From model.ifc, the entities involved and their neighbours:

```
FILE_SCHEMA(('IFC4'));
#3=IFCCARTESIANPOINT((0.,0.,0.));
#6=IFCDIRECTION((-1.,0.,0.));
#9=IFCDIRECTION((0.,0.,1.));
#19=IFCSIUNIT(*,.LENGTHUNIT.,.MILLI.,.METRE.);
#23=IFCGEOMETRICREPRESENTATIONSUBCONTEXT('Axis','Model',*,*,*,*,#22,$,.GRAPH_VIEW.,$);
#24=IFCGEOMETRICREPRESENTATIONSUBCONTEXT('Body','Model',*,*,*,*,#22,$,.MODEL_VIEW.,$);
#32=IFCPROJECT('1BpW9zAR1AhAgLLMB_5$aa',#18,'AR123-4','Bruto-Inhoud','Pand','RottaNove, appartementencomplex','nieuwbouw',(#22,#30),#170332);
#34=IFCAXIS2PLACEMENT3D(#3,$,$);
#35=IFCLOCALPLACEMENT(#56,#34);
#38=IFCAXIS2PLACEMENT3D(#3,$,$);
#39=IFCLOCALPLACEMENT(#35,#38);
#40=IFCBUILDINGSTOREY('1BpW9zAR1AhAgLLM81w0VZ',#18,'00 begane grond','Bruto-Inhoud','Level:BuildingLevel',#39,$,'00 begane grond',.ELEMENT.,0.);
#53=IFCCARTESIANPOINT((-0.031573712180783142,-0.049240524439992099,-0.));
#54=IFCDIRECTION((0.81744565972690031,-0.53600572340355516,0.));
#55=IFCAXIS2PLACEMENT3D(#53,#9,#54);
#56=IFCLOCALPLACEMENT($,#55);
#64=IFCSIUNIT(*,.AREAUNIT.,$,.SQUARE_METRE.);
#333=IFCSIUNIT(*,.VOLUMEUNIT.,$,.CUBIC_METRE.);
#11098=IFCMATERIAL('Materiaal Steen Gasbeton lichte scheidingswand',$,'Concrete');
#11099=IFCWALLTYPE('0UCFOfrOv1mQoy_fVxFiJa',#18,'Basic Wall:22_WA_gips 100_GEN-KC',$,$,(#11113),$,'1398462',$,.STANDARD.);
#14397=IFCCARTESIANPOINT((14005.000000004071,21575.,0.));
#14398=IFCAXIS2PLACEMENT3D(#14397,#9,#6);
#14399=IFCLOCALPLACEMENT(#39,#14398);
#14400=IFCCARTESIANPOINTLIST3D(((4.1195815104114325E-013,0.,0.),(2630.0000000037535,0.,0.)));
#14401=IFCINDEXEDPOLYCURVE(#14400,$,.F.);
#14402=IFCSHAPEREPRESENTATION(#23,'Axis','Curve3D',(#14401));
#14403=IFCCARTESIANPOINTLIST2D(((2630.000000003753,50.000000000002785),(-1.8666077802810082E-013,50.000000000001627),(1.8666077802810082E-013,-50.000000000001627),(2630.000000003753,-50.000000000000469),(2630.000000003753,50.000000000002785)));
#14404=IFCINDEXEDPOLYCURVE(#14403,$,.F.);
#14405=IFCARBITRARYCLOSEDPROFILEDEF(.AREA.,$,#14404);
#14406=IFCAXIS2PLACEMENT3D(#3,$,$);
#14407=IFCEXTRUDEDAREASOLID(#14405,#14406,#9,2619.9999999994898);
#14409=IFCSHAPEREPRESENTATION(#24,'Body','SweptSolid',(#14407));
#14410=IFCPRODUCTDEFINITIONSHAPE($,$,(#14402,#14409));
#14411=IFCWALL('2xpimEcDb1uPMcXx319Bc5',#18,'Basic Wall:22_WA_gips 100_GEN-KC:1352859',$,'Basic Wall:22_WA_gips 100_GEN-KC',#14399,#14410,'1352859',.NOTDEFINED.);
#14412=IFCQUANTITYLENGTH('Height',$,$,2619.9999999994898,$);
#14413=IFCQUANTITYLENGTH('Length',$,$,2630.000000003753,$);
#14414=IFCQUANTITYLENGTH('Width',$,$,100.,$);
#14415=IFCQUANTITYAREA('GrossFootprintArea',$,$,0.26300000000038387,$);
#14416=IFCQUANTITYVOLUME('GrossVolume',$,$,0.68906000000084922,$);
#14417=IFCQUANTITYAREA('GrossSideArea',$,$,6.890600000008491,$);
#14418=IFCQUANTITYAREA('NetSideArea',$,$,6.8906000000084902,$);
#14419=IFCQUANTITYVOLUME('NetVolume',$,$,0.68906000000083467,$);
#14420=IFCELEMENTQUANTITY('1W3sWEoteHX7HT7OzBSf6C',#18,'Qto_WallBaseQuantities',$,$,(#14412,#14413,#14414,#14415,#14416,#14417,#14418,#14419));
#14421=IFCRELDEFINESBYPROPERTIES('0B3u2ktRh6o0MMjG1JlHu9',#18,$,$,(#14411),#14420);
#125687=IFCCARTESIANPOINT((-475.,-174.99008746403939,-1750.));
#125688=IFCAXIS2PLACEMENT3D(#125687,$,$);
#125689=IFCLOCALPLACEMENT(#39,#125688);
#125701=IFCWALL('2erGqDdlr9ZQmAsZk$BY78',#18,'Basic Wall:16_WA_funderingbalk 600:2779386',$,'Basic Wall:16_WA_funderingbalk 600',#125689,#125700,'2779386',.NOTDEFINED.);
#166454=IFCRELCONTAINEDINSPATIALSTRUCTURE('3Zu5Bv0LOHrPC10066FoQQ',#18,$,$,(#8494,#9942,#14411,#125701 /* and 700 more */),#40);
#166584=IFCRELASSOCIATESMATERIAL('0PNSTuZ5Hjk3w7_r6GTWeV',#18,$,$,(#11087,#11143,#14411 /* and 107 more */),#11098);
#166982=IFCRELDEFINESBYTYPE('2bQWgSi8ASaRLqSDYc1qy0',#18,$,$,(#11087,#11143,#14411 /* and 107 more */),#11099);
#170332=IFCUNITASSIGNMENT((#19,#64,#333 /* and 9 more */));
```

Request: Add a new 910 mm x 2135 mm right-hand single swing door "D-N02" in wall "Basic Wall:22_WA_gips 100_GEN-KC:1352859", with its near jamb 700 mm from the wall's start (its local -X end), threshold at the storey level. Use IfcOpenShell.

```python
import numpy as np
import ifcopenshell
import ifcopenshell.api.feature
import ifcopenshell.api.geometry
import ifcopenshell.api.pset
import ifcopenshell.api.root
import ifcopenshell.api.spatial
import ifcopenshell.geom
import ifcopenshell.util.element
import ifcopenshell.util.placement
import ifcopenshell.util.representation
import ifcopenshell.util.shape
import ifcopenshell.util.unit

model = ifcopenshell.open("model.ifc")
unit_scale = ifcopenshell.util.unit.calculate_unit_scale(model)
area_scale = ifcopenshell.util.unit.calculate_unit_scale(model, "AREAUNIT")
volume_scale = ifcopenshell.util.unit.calculate_unit_scale(model, "VOLUMEUNIT")
settings = ifcopenshell.geom.settings()


def volume(element):
    """Net volume in cubic metres, openings subtracted."""
    shape = ifcopenshell.geom.create_shape(settings, element)
    return ifcopenshell.util.shape.get_volume(shape.geometry)


wall = model.by_id(14411)
storey = ifcopenshell.util.element.get_container(wall, ifc_class="IfcBuildingStorey")
context = ifcopenshell.util.representation.get_context(model, "Model", "Body", "MODEL_VIEW")
before = volume(wall)

width, height, from_end, sill = 0.91, 2.135, 0.7, 0.0  # metres

# The wall runs along its own X axis, and the end named is its -X end.
wall_shape = ifcopenshell.geom.create_shape(settings, wall)
x, y, z = ifcopenshell.util.shape.get_vertices(wall_shape.geometry).T
start = x.min() + from_end
face, thickness = float(y.min()), float(y.max() - y.min())
wall_matrix = ifcopenshell.util.placement.get_local_placement(wall.ObjectPlacement)
level = ifcopenshell.util.placement.get_local_placement(storey.ObjectPlacement)[2, 3]


def in_wall(x, y):
    """Placement at x, y metres in the wall's axes, at sill height."""
    matrix = wall_matrix.copy()
    matrix[:, 3] = wall_matrix @ np.array([x / unit_scale, y / unit_scale, 0.0, 1.0])
    matrix[2, 3] = level + sill / unit_scale
    return matrix


# Opening: a box that overshoots both wall faces by 50 mm.
opening = ifcopenshell.api.root.create_entity(model, ifc_class="IfcOpeningElement", predefined_type="OPENING")
box = ifcopenshell.api.geometry.add_wall_representation(
    model, context=context, length=width, height=height, thickness=thickness + 0.1
)
ifcopenshell.api.geometry.assign_representation(model, product=opening, representation=box)
ifcopenshell.api.geometry.edit_object_placement(model, product=opening, matrix=in_wall(start, face - 0.05), is_si=False)
ifcopenshell.api.feature.add_feature(model, feature=opening, element=wall)

door = ifcopenshell.api.root.create_entity(model, ifc_class="IfcDoor", name="D-N02", predefined_type="DOOR")
door.OverallWidth, door.OverallHeight = width / unit_scale, height / unit_scale
door.OperationType = "SINGLE_SWING_RIGHT"
body = ifcopenshell.api.geometry.add_door_representation(
    model,
    context=context,
    overall_width=door.OverallWidth,
    overall_height=door.OverallHeight,
    operation_type="SINGLE_SWING_RIGHT",
    lining_properties={"LiningDepth": thickness / unit_scale, "ThresholdDepth": thickness / unit_scale},
)
ifcopenshell.api.geometry.assign_representation(model, product=door, representation=body)
ifcopenshell.api.spatial.assign_container(model, products=[door], relating_structure=storey)
ifcopenshell.api.feature.add_filling(model, opening=opening, element=door)

# The lining spans the wall, so the door starts at the wall face.
ifcopenshell.api.geometry.edit_object_placement(model, product=door, matrix=in_wall(start, face), is_si=False)

after = volume(wall)

# Update the wall's stored quantities.
qto = model.by_id(ifcopenshell.util.element.get_pset(wall, "Qto_WallBaseQuantities", should_inherit=False)["id"])
ifcopenshell.api.pset.edit_qto(model, qto=qto, properties={
    "NetSideArea": after / thickness / area_scale,
    "NetVolume": after / volume_scale,
})

print(f"wall volume {before:.3f} -> {after:.3f} m3")

model.write("model_updated.ifc")
```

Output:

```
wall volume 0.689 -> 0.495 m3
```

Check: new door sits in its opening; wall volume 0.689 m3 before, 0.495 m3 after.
